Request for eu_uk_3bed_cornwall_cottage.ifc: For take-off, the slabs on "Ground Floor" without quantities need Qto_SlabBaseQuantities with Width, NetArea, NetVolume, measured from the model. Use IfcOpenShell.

First a look at what the model holds.

```python
import ifcopenshell
import ifcopenshell.util.element
import ifcopenshell.util.unit

model = ifcopenshell.open("eu_uk_3bed_cornwall_cottage.ifc")
print(model.schema)
for unit_type in ("LENGTHUNIT", "AREAUNIT", "VOLUMEUNIT"):
    print(unit_type, ifcopenshell.util.unit.calculate_unit_scale(model, unit_type))
storey = next(s for s in model.by_type("IfcBuildingStorey") if s.Name == "Ground Floor")
slabs = [e for e in ifcopenshell.util.element.get_decomposition(storey) if e.is_a("IfcSlab")]
for e in sorted(slabs, key=lambda e: e.id()):
    print(e.id(), e.is_a(), e.Name, list(ifcopenshell.util.element.get_psets(e, qtos_only=True)), sep=" | ")
```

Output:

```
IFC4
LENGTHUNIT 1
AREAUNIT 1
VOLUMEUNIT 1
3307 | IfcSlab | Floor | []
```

```python
import ifcopenshell
import ifcopenshell.api.pset
import ifcopenshell.geom
import ifcopenshell.util.element
import ifcopenshell.util.shape
import ifcopenshell.util.unit

model = ifcopenshell.open("eu_uk_3bed_cornwall_cottage.ifc")
unit_scale = ifcopenshell.util.unit.calculate_unit_scale(model)
area_scale = ifcopenshell.util.unit.calculate_unit_scale(model, "AREAUNIT")
volume_scale = ifcopenshell.util.unit.calculate_unit_scale(model, "VOLUMEUNIT")
settings = ifcopenshell.geom.settings()

storey = next(s for s in model.by_type("IfcBuildingStorey") if s.Name == "Ground Floor")
slabs = [e for e in ifcopenshell.util.element.get_decomposition(storey) if e.is_a("IfcSlab")]

for e in sorted(slabs, key=lambda e: e.id()):
    if ifcopenshell.util.element.get_psets(e, qtos_only=True, should_inherit=False):
        continue
    # Geometry comes back in metres, in the element's own axes.
    shape = ifcopenshell.geom.create_shape(settings, e)
    values = {
        "Width": ifcopenshell.util.shape.get_z(shape.geometry) / unit_scale,
        "NetArea": ifcopenshell.util.shape.get_footprint_area(shape.geometry) / area_scale,
        "NetVolume": ifcopenshell.util.shape.get_volume(shape.geometry) / volume_scale,
    }
    qto = ifcopenshell.api.pset.add_qto(model, product=e, name="Qto_SlabBaseQuantities")
    ifcopenshell.api.pset.edit_qto(model, qto=qto, properties=values)
    print(e.id(), {k: round(v, 3) for k, v in values.items()})

model.write("eu_uk_3bed_cornwall_cottage_v2.ifc")
```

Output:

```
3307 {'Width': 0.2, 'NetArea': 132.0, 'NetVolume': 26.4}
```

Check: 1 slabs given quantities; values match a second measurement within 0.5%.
